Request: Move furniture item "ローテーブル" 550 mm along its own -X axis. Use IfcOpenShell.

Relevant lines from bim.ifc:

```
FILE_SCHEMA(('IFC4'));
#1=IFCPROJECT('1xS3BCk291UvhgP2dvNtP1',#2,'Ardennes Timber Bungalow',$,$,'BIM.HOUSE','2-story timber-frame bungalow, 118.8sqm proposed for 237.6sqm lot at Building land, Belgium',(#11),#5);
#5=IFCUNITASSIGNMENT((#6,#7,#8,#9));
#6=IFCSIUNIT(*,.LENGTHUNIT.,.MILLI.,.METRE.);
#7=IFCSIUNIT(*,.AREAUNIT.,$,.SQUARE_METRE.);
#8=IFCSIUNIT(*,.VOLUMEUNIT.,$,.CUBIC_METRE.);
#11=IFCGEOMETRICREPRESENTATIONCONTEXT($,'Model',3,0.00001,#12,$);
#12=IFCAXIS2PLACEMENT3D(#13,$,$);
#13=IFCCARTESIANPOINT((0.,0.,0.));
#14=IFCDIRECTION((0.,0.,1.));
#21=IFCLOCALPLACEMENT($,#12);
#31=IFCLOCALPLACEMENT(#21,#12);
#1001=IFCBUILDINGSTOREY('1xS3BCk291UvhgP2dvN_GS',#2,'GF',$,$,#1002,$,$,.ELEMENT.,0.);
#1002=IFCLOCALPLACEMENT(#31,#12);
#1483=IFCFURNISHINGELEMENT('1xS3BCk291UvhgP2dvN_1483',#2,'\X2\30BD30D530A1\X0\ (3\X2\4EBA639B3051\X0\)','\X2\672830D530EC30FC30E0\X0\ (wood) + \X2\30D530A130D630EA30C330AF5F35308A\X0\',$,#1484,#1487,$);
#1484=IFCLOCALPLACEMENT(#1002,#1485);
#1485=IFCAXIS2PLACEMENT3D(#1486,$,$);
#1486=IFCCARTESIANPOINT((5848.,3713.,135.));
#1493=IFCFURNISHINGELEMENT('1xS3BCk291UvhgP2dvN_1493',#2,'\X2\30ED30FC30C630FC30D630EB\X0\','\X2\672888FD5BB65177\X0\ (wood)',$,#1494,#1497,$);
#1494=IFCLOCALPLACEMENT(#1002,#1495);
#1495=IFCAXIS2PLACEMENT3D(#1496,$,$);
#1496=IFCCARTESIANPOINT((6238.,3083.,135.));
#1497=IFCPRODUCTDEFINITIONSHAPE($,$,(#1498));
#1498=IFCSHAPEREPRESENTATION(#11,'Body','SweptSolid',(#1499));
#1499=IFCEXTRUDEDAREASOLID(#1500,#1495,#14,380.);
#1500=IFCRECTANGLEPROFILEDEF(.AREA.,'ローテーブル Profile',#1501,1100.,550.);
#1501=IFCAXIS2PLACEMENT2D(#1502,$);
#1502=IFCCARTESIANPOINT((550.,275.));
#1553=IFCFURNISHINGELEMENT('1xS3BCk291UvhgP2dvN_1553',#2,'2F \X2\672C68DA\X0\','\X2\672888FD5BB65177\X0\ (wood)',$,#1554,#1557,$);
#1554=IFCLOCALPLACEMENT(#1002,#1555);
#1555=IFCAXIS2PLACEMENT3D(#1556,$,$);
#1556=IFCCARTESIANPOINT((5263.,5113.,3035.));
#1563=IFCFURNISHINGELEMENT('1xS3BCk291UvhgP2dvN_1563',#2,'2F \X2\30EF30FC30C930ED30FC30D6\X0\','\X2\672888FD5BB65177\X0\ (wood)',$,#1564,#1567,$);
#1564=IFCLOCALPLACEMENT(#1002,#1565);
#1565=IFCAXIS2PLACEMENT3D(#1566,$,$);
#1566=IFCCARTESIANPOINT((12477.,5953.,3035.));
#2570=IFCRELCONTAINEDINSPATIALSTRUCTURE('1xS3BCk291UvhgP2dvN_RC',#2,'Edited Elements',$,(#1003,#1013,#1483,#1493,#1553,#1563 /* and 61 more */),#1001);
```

```python
import ifcopenshell
import ifcopenshell.api.geometry
import ifcopenshell.util.placement

model = ifcopenshell.open("bim.ifc")

item = model.by_id(1493)
matrix = ifcopenshell.util.placement.get_local_placement(item.ObjectPlacement)
matrix[:3, 3] -= matrix[:3, 0] * 550.0
ifcopenshell.api.geometry.edit_object_placement(model, product=item, matrix=matrix, is_si=False)

print(ifcopenshell.util.placement.get_local_placement(item.ObjectPlacement).round(3) + 0.0)

model.write("bim_rev.ifc")
```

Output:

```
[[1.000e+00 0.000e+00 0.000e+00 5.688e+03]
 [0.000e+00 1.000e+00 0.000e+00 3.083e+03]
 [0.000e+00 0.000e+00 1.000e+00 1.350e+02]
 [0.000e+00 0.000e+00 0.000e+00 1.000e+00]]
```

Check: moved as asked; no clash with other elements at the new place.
